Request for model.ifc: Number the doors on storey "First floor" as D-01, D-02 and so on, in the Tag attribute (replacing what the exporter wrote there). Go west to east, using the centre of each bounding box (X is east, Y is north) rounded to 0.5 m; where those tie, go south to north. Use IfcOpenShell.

First a look at what the model holds.

```python
import ifcopenshell
import ifcopenshell.util.element
import ifcopenshell.util.placement

model = ifcopenshell.open("model.ifc")
print(model.schema)
storey = next(s for s in model.by_type("IfcBuildingStorey") if s.Name == "First floor")
doors = [e for e in ifcopenshell.util.element.get_decomposition(storey) if e.is_a("IfcDoor")]
for e in sorted(doors, key=lambda e: e.id()):
    origin = ifcopenshell.util.placement.get_local_placement(e.ObjectPlacement)[:3, 3]
    print(e.id(), e.Tag, e.Name, origin.round(2) + 0.0, sep=" | ")
```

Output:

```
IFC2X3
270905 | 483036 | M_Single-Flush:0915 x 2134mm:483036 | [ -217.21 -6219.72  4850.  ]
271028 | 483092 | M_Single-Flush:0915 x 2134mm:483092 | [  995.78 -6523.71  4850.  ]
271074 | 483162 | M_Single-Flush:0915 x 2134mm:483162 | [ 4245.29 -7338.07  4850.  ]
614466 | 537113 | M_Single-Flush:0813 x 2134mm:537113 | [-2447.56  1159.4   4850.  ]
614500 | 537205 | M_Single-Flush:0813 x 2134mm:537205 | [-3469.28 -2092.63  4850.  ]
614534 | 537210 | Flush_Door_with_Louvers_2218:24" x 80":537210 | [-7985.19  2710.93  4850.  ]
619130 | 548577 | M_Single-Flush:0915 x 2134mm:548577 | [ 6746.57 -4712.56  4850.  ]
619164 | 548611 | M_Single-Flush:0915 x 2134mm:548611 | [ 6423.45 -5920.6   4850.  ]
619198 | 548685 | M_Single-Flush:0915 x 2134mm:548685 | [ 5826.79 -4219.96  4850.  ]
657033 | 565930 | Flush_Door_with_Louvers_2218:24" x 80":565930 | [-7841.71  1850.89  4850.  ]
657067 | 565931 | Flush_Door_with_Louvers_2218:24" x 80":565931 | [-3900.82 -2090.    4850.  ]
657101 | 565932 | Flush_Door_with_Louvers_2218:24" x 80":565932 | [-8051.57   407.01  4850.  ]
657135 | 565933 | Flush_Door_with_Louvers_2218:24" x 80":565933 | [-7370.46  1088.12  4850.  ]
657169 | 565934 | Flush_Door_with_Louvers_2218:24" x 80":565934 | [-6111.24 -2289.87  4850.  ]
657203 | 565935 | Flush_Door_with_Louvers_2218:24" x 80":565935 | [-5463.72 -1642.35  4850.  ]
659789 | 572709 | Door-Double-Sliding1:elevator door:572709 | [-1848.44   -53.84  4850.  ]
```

```python
import ifcopenshell
import ifcopenshell.geom
import ifcopenshell.util.element
import ifcopenshell.util.shape

model = ifcopenshell.open("model.ifc")
settings = ifcopenshell.geom.settings()
settings.set("use-world-coords", True)


def centre(element):
    shape = ifcopenshell.geom.create_shape(settings, element)
    return ifcopenshell.util.shape.get_bbox_centroid(shape.geometry)


storey = next(s for s in model.by_type("IfcBuildingStorey") if s.Name == "First floor")
doors = [e for e in ifcopenshell.util.element.get_decomposition(storey) if e.is_a("IfcDoor")]

# Insertion points can sit at a corner or the storey origin, so sort by the geometry (in metres).
centres = {e: centre(e) for e in doors}
doors.sort(key=lambda e: (round(centres[e][0] / 0.5), centres[e][1]))

for i, e in enumerate(doors, start=1):
    number = f"D-{i:02d}"
    e.Tag = number
    print(e.id(), number)

model.write("model-out.ifc")
```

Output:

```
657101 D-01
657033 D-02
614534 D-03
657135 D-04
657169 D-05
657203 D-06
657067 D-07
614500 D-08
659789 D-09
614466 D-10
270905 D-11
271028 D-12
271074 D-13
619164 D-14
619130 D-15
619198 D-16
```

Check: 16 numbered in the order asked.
